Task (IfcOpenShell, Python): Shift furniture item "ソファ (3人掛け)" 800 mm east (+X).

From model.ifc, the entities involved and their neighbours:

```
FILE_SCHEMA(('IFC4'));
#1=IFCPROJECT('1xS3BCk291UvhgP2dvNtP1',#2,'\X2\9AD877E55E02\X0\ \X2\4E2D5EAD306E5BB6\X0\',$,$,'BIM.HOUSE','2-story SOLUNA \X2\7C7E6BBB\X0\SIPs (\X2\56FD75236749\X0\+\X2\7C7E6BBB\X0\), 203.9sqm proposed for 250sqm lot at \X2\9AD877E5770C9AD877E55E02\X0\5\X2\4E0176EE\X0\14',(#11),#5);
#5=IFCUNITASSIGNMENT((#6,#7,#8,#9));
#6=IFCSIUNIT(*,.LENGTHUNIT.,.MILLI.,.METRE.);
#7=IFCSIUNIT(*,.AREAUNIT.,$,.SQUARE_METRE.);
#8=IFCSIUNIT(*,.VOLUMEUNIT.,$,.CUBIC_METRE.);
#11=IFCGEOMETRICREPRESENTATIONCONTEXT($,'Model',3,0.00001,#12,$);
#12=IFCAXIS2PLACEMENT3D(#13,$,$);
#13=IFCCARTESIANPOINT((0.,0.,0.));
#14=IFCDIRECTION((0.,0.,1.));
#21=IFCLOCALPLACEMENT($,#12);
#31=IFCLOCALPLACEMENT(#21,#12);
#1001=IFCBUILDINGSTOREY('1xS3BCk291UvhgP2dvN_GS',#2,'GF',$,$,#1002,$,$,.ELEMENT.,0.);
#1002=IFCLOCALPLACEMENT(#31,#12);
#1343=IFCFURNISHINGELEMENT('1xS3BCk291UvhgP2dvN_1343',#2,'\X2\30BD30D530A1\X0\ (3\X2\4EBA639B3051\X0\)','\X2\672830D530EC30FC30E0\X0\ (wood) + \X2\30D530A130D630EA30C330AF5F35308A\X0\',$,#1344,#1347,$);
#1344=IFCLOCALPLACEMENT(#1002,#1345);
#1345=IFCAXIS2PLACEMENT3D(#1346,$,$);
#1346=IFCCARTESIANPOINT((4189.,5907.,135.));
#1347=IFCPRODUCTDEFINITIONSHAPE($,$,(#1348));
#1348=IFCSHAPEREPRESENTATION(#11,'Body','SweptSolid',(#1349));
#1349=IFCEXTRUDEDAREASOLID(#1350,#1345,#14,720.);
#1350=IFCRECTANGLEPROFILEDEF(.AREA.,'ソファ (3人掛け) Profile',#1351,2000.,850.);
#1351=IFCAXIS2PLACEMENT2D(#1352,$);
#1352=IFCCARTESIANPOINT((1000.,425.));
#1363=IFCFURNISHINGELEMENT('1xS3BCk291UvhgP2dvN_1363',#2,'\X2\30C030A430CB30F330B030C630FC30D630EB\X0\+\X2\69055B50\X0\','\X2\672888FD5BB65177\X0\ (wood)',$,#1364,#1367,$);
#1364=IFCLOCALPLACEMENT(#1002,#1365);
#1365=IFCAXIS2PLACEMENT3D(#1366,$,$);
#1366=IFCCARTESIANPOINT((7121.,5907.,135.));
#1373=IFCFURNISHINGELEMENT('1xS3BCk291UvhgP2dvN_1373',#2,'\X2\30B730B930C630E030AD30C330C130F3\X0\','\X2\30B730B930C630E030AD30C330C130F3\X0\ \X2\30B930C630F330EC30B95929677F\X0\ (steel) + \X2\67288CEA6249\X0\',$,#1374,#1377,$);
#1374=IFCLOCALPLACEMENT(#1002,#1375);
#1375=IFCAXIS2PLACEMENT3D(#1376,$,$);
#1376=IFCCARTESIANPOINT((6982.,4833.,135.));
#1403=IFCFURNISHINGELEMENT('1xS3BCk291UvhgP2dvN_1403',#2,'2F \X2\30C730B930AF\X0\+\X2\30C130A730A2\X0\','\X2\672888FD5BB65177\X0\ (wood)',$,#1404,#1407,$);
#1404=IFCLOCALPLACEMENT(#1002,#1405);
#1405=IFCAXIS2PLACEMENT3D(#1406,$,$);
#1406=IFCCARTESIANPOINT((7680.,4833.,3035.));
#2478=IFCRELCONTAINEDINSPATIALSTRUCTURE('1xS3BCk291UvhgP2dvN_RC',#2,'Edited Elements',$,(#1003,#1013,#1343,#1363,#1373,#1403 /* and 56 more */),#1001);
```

```python
import ifcopenshell
import ifcopenshell.api.geometry
import ifcopenshell.util.placement

model = ifcopenshell.open("model.ifc")

item = model.by_id(1343)
matrix = ifcopenshell.util.placement.get_local_placement(item.ObjectPlacement)
matrix[0, 3] += 800.0
ifcopenshell.api.geometry.edit_object_placement(model, product=item, matrix=matrix, is_si=False)

print(ifcopenshell.util.placement.get_local_placement(item.ObjectPlacement).round(3) + 0.0)

model.write("model_v2.ifc")
```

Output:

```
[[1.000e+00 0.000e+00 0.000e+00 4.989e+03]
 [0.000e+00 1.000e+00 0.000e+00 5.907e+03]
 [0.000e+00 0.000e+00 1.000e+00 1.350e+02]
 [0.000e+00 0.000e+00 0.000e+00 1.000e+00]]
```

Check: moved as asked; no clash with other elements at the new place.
